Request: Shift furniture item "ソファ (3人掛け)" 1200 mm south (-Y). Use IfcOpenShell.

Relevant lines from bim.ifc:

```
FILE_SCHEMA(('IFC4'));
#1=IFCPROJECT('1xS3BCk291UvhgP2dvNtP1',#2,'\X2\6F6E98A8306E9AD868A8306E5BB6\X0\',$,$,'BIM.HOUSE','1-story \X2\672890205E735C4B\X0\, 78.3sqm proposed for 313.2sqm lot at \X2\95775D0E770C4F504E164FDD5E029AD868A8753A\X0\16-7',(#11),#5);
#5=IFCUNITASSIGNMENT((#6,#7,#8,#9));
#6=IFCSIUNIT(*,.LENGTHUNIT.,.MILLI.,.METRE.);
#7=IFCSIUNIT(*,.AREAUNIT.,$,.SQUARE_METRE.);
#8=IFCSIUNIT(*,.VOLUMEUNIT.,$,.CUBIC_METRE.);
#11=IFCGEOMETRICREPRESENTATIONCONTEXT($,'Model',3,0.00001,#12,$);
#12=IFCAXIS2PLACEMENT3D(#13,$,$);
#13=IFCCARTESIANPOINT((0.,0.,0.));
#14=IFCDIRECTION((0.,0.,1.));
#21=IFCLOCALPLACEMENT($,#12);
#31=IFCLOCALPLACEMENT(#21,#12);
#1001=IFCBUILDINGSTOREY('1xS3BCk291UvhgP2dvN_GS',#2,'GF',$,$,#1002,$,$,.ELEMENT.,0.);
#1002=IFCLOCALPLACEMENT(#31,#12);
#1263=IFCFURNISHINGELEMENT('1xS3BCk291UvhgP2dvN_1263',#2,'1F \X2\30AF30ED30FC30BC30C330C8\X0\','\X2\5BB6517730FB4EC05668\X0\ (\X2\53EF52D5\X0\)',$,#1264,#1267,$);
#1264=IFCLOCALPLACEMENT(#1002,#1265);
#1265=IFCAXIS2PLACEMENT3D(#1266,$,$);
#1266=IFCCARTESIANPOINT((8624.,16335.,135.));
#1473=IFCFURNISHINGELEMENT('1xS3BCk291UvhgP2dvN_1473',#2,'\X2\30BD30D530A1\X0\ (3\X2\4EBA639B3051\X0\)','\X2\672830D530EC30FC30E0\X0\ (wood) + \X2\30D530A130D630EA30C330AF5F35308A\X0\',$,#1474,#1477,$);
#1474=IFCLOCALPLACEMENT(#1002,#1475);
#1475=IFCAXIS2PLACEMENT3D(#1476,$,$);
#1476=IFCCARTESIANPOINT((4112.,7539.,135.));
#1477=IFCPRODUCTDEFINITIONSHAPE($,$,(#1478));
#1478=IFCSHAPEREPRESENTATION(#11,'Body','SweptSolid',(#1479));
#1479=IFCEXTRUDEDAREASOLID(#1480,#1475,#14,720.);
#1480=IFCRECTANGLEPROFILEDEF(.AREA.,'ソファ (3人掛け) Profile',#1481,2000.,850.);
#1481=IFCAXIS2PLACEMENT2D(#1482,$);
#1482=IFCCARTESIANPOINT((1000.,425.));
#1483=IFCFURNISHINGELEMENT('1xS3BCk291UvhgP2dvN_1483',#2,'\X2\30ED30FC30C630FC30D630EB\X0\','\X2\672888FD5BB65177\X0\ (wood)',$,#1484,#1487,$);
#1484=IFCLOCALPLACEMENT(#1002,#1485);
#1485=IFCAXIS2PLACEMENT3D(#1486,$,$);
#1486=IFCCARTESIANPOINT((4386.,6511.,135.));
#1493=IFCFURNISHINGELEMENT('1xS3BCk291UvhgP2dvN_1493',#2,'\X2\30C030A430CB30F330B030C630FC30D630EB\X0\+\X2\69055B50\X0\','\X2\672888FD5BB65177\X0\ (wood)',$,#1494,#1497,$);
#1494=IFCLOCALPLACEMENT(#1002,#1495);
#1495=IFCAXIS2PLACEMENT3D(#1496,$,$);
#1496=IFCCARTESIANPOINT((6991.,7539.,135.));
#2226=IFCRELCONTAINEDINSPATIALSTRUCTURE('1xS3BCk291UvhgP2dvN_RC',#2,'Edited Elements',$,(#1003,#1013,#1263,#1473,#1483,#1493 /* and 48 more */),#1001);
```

```python
import ifcopenshell
import ifcopenshell.api.geometry
import ifcopenshell.util.placement

model = ifcopenshell.open("bim.ifc")

item = model.by_guid("1xS3BCk291UvhgP2dvN_1473")
matrix = ifcopenshell.util.placement.get_local_placement(item.ObjectPlacement)
matrix[1, 3] -= 1200.0
ifcopenshell.api.geometry.edit_object_placement(model, product=item, matrix=matrix, is_si=False)

print(ifcopenshell.util.placement.get_local_placement(item.ObjectPlacement).round(3) + 0.0)

model.write("bim_updated.ifc")
```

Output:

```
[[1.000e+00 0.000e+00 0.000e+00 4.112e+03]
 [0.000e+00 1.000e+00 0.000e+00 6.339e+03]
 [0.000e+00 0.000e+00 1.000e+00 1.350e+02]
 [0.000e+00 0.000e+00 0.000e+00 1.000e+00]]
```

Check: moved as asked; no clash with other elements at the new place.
